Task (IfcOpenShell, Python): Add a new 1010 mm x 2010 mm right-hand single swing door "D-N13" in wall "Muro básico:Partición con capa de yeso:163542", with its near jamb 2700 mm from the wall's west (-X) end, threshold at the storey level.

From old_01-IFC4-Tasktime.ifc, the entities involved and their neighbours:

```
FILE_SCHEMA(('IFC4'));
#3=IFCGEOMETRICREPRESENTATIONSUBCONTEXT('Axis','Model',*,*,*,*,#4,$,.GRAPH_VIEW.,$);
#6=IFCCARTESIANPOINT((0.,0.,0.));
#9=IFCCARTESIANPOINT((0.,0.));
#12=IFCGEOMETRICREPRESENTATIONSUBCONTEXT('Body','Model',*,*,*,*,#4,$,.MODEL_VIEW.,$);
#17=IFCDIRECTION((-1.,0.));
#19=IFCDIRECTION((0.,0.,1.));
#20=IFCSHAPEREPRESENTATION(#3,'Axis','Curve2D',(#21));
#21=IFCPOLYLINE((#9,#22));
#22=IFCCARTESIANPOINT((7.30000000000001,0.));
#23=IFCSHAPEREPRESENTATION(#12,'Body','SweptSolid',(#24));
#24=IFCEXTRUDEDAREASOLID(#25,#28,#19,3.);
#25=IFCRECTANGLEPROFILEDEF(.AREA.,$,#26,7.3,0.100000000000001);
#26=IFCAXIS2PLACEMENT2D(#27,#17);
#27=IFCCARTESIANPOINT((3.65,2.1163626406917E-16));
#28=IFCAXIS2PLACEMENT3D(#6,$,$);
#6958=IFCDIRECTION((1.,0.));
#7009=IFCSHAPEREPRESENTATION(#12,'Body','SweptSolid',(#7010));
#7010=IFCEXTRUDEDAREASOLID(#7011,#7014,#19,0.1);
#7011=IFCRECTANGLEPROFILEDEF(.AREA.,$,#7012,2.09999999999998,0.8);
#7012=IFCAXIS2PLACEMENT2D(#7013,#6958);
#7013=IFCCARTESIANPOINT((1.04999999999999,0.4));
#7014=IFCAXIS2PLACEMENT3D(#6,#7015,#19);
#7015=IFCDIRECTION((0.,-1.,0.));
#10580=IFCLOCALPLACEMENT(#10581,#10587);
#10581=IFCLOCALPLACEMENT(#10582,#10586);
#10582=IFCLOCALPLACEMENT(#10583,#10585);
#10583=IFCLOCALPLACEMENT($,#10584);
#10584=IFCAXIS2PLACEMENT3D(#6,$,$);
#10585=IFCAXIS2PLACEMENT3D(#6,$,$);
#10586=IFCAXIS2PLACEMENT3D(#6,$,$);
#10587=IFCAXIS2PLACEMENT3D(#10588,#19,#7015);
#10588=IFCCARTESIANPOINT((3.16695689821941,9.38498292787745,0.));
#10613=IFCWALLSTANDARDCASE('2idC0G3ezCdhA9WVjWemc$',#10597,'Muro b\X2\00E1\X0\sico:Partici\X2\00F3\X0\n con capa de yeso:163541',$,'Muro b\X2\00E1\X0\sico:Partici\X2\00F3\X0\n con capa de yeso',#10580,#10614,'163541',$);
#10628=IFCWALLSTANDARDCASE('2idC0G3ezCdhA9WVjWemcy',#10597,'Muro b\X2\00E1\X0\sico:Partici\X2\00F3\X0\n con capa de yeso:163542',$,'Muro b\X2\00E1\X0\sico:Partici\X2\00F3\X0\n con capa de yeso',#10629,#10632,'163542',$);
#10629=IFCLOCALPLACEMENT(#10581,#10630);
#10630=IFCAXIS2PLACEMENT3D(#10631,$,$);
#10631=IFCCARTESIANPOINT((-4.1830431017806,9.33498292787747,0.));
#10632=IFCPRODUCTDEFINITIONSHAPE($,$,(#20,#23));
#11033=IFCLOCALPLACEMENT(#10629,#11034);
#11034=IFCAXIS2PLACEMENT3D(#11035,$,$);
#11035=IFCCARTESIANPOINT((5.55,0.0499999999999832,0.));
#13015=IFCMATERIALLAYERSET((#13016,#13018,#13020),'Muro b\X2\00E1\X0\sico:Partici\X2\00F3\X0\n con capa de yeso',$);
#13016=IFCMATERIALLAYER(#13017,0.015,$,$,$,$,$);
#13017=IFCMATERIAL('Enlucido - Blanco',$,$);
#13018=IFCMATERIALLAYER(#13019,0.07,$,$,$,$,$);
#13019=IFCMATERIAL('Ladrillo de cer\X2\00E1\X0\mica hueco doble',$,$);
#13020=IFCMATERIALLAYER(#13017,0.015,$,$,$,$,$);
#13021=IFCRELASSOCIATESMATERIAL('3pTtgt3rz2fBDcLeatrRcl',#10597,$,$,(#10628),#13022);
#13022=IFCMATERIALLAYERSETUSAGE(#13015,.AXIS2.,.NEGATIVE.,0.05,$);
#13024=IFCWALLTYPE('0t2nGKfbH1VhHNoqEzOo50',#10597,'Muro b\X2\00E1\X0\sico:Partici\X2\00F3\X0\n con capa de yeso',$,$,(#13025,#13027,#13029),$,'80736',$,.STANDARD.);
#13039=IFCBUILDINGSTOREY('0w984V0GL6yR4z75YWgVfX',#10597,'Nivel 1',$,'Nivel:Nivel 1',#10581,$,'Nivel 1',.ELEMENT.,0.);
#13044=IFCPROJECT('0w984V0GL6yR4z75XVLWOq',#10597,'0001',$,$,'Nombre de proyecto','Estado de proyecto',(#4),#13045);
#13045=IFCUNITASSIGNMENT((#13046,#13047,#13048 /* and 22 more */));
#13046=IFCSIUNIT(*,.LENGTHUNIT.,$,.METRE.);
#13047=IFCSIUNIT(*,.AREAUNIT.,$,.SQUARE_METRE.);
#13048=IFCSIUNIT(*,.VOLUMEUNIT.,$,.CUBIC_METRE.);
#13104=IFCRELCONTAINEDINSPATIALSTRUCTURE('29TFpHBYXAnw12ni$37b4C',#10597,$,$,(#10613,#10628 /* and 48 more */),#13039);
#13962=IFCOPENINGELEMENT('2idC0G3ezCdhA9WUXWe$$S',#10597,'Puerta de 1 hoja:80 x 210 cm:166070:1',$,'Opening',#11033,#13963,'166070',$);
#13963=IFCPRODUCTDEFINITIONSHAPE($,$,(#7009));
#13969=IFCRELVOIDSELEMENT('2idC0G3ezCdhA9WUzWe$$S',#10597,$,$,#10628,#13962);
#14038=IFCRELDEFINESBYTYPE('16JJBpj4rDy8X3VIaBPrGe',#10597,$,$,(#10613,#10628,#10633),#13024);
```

```python
import numpy as np
import ifcopenshell
import ifcopenshell.api.feature
import ifcopenshell.api.geometry
import ifcopenshell.api.root
import ifcopenshell.api.spatial
import ifcopenshell.geom
import ifcopenshell.util.element
import ifcopenshell.util.placement
import ifcopenshell.util.representation
import ifcopenshell.util.shape
import ifcopenshell.util.unit

model = ifcopenshell.open("old_01-IFC4-Tasktime.ifc")
unit_scale = ifcopenshell.util.unit.calculate_unit_scale(model)
settings = ifcopenshell.geom.settings()


def volume(element):
    """Net volume in cubic metres, openings subtracted."""
    shape = ifcopenshell.geom.create_shape(settings, element)
    return ifcopenshell.util.shape.get_volume(shape.geometry)


wall = model.by_id(10628)
storey = ifcopenshell.util.element.get_container(wall, ifc_class="IfcBuildingStorey")
context = ifcopenshell.util.representation.get_context(model, "Model", "Body", "MODEL_VIEW")
before = volume(wall)

width, height, from_end, sill = 1.01, 2.01, 2.7, 0.0  # metres

# The wall runs along its own X axis, and the end named is its -X end.
wall_shape = ifcopenshell.geom.create_shape(settings, wall)
x, y, z = ifcopenshell.util.shape.get_vertices(wall_shape.geometry).T
start = x.min() + from_end
face, thickness = float(y.min()), float(y.max() - y.min())
wall_matrix = ifcopenshell.util.placement.get_local_placement(wall.ObjectPlacement)
level = ifcopenshell.util.placement.get_local_placement(storey.ObjectPlacement)[2, 3]


def in_wall(x, y):
    """Placement at x, y metres in the wall's axes, at sill height."""
    matrix = wall_matrix.copy()
    matrix[:, 3] = wall_matrix @ np.array([x / unit_scale, y / unit_scale, 0.0, 1.0])
    matrix[2, 3] = level + sill / unit_scale
    return matrix


# Opening: a box that overshoots both wall faces by 50 mm.
opening = ifcopenshell.api.root.create_entity(model, ifc_class="IfcOpeningElement", predefined_type="OPENING")
box = ifcopenshell.api.geometry.add_wall_representation(
    model, context=context, length=width, height=height, thickness=thickness + 0.1
)
ifcopenshell.api.geometry.assign_representation(model, product=opening, representation=box)
ifcopenshell.api.geometry.edit_object_placement(model, product=opening, matrix=in_wall(start, face - 0.05), is_si=False)
ifcopenshell.api.feature.add_feature(model, feature=opening, element=wall)

door = ifcopenshell.api.root.create_entity(model, ifc_class="IfcDoor", name="D-N13", predefined_type="DOOR")
door.OverallWidth, door.OverallHeight = width / unit_scale, height / unit_scale
door.OperationType = "SINGLE_SWING_RIGHT"
body = ifcopenshell.api.geometry.add_door_representation(
    model,
    context=context,
    overall_width=door.OverallWidth,
    overall_height=door.OverallHeight,
    operation_type="SINGLE_SWING_RIGHT",
    lining_properties={"LiningDepth": thickness / unit_scale, "ThresholdDepth": thickness / unit_scale},
)
ifcopenshell.api.geometry.assign_representation(model, product=door, representation=body)
ifcopenshell.api.spatial.assign_container(model, products=[door], relating_structure=storey)
ifcopenshell.api.feature.add_filling(model, opening=opening, element=door)

# The lining spans the wall, so the door starts at the wall face.
ifcopenshell.api.geometry.edit_object_placement(model, product=door, matrix=in_wall(start, face), is_si=False)

after = volume(wall)

print(f"wall volume {before:.3f} -> {after:.3f} m3")

model.write("old_01-IFC4-Tasktime_edited.ifc")
```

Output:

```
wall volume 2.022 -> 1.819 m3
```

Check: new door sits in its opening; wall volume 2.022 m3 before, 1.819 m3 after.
